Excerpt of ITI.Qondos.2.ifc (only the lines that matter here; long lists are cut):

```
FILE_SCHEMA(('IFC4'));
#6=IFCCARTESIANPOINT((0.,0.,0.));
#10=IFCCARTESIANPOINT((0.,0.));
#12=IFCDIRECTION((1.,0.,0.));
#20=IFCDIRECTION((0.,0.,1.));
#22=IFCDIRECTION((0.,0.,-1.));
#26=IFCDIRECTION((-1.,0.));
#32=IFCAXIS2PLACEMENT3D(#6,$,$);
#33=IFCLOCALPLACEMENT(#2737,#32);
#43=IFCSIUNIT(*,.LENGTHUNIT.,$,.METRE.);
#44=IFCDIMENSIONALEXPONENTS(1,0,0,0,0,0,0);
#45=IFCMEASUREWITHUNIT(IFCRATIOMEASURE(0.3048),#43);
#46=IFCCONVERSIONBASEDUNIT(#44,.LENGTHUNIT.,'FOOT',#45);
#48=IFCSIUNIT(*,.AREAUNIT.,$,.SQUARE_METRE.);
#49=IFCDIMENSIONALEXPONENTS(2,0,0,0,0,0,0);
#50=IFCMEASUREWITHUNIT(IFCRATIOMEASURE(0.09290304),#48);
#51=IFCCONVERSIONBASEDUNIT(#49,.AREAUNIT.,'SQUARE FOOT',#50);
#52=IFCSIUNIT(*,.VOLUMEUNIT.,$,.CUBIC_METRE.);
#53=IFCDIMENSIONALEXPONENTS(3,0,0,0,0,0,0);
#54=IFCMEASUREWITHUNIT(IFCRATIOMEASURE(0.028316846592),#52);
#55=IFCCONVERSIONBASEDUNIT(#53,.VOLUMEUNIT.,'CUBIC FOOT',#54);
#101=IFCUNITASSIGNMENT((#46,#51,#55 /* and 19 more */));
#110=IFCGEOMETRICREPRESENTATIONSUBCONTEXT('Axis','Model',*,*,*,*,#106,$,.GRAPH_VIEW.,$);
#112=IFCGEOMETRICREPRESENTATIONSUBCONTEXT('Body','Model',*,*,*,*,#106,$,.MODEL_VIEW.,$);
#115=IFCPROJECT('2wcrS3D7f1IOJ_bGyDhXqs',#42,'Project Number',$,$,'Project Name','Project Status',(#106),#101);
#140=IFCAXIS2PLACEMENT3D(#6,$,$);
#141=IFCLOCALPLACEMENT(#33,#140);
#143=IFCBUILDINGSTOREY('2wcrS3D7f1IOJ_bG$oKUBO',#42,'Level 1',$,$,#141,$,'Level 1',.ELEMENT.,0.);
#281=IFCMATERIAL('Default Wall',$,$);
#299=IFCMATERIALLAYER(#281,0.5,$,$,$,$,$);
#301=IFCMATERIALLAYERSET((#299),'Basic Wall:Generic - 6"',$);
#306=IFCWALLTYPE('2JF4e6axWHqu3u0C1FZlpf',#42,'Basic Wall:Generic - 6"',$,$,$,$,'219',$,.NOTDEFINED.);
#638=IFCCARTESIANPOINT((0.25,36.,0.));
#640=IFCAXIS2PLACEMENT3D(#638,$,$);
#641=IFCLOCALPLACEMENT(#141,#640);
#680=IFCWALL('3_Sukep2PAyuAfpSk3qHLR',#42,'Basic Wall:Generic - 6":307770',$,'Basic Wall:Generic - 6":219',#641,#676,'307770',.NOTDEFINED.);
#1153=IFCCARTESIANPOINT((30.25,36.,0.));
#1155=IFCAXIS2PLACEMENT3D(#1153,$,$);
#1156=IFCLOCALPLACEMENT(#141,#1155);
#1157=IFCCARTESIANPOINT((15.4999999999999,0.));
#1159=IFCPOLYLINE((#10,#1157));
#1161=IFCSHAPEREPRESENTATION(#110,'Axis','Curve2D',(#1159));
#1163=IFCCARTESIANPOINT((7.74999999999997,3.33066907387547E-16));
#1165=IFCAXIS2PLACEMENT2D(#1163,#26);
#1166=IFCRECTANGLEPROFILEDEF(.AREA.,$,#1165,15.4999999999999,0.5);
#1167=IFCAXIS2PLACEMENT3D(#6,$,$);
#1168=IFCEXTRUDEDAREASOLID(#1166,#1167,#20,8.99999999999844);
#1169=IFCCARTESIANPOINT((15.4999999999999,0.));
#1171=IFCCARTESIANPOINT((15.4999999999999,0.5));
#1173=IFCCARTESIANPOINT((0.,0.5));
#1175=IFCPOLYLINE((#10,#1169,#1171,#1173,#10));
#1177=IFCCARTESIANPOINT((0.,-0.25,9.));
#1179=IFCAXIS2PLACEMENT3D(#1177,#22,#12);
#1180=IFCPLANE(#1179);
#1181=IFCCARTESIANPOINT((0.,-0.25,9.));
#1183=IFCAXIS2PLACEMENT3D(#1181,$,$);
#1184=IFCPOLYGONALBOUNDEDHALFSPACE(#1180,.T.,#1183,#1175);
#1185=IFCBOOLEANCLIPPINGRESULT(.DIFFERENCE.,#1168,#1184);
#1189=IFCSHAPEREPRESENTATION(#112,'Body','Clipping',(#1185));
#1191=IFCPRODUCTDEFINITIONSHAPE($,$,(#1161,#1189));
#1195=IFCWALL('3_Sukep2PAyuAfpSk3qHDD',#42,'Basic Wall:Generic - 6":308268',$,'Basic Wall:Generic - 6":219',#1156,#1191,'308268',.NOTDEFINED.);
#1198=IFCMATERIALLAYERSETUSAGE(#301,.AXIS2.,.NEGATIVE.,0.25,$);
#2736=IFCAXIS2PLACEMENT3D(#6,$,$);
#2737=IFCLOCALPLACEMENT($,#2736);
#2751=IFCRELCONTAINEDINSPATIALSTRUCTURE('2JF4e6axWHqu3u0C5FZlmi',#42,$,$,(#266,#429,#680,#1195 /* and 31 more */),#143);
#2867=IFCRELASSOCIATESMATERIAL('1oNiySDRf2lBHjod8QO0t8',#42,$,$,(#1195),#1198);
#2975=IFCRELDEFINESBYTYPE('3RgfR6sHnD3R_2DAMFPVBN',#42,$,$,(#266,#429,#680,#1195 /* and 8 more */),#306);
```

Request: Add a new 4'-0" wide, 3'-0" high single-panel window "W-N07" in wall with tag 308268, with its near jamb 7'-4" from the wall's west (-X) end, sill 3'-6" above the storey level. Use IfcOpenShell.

```python
import numpy as np
import ifcopenshell
import ifcopenshell.api.feature
import ifcopenshell.api.geometry
import ifcopenshell.api.root
import ifcopenshell.api.spatial
import ifcopenshell.geom
import ifcopenshell.util.element
import ifcopenshell.util.placement
import ifcopenshell.util.representation
import ifcopenshell.util.shape
import ifcopenshell.util.unit

model = ifcopenshell.open("ITI.Qondos.2.ifc")
unit_scale = ifcopenshell.util.unit.calculate_unit_scale(model)
settings = ifcopenshell.geom.settings()


def volume(element):
    """Net volume in cubic metres, openings subtracted."""
    shape = ifcopenshell.geom.create_shape(settings, element)
    return ifcopenshell.util.shape.get_volume(shape.geometry)


wall = model.by_guid("3_Sukep2PAyuAfpSk3qHDD")
storey = ifcopenshell.util.element.get_container(wall, ifc_class="IfcBuildingStorey")
context = ifcopenshell.util.representation.get_context(model, "Model", "Body", "MODEL_VIEW")
before = volume(wall)

width, height, from_end, sill = 1.2192, 0.9144, 2.2352, 1.0668  # metres

# The wall runs along its own X axis, and the end named is its -X end.
wall_shape = ifcopenshell.geom.create_shape(settings, wall)
x, y, z = ifcopenshell.util.shape.get_vertices(wall_shape.geometry).T
start = x.min() + from_end
face, thickness = float(y.min()), float(y.max() - y.min())
wall_matrix = ifcopenshell.util.placement.get_local_placement(wall.ObjectPlacement)
level = ifcopenshell.util.placement.get_local_placement(storey.ObjectPlacement)[2, 3]


def in_wall(x, y):
    """Placement at x, y metres in the wall's axes, at sill height."""
    matrix = wall_matrix.copy()
    matrix[:, 3] = wall_matrix @ np.array([x / unit_scale, y / unit_scale, 0.0, 1.0])
    matrix[2, 3] = level + sill / unit_scale
    return matrix


# Opening: a box that overshoots both wall faces by 50 mm.
opening = ifcopenshell.api.root.create_entity(model, ifc_class="IfcOpeningElement", predefined_type="OPENING")
box = ifcopenshell.api.geometry.add_wall_representation(
    model, context=context, length=width, height=height, thickness=thickness + 0.1
)
ifcopenshell.api.geometry.assign_representation(model, product=opening, representation=box)
ifcopenshell.api.geometry.edit_object_placement(model, product=opening, matrix=in_wall(start, face - 0.05), is_si=False)
ifcopenshell.api.feature.add_feature(model, feature=opening, element=wall)

window = ifcopenshell.api.root.create_entity(model, ifc_class="IfcWindow", name="W-N07", predefined_type="WINDOW")
window.OverallWidth, window.OverallHeight = width / unit_scale, height / unit_scale
window.PartitioningType = "SINGLE_PANEL"
body = ifcopenshell.api.geometry.add_window_representation(
    model,
    context=context,
    overall_width=window.OverallWidth,
    overall_height=window.OverallHeight,
    partition_type="SINGLE_PANEL",
)
ifcopenshell.api.geometry.assign_representation(model, product=window, representation=body)
ifcopenshell.api.spatial.assign_container(model, products=[window], relating_structure=storey)
ifcopenshell.api.feature.add_filling(model, opening=opening, element=window)

# Centre the window in the wall's thickness.
ifcopenshell.api.geometry.edit_object_placement(model, product=window, matrix=in_wall(start, face), is_si=False)
window_shape = ifcopenshell.geom.create_shape(settings, window)
depth = ifcopenshell.util.shape.get_vertices(window_shape.geometry)[:, 1]
offset = face + thickness / 2 - (depth.min() + depth.max()) / 2
ifcopenshell.api.geometry.edit_object_placement(model, product=window, matrix=in_wall(start, offset), is_si=False)

after = volume(wall)

print(f"wall volume {before:.3f} -> {after:.3f} m3")

model.write("ITI.Qondos.2_edited.ifc")
```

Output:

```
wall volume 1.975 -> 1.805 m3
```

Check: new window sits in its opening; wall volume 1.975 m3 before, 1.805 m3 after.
